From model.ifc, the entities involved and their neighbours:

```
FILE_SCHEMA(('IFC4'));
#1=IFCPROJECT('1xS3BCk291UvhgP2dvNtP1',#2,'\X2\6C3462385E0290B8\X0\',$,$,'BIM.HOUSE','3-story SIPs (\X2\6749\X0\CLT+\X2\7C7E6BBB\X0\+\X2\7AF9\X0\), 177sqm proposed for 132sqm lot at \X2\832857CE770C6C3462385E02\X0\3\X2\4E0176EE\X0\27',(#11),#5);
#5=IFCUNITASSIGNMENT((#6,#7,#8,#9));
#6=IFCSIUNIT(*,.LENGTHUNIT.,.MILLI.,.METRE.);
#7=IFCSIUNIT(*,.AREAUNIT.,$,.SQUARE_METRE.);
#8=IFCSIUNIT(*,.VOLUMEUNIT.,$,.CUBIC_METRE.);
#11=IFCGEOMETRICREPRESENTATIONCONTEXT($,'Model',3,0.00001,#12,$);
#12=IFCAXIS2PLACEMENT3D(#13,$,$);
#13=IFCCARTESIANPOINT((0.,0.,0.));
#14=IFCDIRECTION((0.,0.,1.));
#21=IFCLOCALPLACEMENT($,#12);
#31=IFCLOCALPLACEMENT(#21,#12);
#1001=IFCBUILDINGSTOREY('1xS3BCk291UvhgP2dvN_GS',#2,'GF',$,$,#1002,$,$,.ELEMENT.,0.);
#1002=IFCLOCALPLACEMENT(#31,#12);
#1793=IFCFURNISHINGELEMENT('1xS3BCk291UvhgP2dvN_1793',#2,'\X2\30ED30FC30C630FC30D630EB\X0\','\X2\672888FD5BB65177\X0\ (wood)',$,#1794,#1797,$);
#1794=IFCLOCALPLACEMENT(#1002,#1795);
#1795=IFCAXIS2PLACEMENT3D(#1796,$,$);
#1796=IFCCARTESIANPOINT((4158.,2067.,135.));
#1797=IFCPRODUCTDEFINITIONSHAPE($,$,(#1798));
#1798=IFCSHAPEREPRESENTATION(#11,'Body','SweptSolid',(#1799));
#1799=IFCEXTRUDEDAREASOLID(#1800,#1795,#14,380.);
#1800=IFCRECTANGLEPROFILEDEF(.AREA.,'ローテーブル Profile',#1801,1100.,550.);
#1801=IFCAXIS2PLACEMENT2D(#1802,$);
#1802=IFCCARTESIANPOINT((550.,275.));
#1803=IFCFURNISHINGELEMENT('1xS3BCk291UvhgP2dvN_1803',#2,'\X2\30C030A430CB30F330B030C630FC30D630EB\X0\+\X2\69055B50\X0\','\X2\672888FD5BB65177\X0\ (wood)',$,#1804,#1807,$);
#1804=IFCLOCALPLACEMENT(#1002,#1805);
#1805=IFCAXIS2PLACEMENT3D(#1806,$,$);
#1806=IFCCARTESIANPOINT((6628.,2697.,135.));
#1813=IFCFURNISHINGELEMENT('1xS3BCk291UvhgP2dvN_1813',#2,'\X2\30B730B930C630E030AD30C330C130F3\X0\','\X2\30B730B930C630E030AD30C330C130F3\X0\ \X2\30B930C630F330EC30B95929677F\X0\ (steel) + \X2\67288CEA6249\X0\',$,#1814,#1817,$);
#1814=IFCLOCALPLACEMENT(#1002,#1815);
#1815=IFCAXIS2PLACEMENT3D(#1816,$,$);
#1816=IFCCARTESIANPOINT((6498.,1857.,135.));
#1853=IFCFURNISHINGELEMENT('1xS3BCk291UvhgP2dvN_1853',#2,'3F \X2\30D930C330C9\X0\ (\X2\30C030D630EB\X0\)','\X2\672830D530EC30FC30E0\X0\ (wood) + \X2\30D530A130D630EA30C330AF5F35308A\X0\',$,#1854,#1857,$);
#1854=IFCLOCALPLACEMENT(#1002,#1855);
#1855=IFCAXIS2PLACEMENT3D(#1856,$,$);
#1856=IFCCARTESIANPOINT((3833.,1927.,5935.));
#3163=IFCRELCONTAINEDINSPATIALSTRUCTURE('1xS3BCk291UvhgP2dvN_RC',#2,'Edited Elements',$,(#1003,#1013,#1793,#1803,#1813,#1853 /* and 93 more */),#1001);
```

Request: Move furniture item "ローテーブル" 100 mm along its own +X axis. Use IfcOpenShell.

```python
import ifcopenshell
import ifcopenshell.api.geometry
import ifcopenshell.util.placement

model = ifcopenshell.open("model.ifc")

item = model.by_guid("1xS3BCk291UvhgP2dvN_1793")
matrix = ifcopenshell.util.placement.get_local_placement(item.ObjectPlacement)
matrix[:3, 3] += matrix[:3, 0] * 100.0
ifcopenshell.api.geometry.edit_object_placement(model, product=item, matrix=matrix, is_si=False)

print(ifcopenshell.util.placement.get_local_placement(item.ObjectPlacement).round(3) + 0.0)

model.write("model_v2.ifc")
```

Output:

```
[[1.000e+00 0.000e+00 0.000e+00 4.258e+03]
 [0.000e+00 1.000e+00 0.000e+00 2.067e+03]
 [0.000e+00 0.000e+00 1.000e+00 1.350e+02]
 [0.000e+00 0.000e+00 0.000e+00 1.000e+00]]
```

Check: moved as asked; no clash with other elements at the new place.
